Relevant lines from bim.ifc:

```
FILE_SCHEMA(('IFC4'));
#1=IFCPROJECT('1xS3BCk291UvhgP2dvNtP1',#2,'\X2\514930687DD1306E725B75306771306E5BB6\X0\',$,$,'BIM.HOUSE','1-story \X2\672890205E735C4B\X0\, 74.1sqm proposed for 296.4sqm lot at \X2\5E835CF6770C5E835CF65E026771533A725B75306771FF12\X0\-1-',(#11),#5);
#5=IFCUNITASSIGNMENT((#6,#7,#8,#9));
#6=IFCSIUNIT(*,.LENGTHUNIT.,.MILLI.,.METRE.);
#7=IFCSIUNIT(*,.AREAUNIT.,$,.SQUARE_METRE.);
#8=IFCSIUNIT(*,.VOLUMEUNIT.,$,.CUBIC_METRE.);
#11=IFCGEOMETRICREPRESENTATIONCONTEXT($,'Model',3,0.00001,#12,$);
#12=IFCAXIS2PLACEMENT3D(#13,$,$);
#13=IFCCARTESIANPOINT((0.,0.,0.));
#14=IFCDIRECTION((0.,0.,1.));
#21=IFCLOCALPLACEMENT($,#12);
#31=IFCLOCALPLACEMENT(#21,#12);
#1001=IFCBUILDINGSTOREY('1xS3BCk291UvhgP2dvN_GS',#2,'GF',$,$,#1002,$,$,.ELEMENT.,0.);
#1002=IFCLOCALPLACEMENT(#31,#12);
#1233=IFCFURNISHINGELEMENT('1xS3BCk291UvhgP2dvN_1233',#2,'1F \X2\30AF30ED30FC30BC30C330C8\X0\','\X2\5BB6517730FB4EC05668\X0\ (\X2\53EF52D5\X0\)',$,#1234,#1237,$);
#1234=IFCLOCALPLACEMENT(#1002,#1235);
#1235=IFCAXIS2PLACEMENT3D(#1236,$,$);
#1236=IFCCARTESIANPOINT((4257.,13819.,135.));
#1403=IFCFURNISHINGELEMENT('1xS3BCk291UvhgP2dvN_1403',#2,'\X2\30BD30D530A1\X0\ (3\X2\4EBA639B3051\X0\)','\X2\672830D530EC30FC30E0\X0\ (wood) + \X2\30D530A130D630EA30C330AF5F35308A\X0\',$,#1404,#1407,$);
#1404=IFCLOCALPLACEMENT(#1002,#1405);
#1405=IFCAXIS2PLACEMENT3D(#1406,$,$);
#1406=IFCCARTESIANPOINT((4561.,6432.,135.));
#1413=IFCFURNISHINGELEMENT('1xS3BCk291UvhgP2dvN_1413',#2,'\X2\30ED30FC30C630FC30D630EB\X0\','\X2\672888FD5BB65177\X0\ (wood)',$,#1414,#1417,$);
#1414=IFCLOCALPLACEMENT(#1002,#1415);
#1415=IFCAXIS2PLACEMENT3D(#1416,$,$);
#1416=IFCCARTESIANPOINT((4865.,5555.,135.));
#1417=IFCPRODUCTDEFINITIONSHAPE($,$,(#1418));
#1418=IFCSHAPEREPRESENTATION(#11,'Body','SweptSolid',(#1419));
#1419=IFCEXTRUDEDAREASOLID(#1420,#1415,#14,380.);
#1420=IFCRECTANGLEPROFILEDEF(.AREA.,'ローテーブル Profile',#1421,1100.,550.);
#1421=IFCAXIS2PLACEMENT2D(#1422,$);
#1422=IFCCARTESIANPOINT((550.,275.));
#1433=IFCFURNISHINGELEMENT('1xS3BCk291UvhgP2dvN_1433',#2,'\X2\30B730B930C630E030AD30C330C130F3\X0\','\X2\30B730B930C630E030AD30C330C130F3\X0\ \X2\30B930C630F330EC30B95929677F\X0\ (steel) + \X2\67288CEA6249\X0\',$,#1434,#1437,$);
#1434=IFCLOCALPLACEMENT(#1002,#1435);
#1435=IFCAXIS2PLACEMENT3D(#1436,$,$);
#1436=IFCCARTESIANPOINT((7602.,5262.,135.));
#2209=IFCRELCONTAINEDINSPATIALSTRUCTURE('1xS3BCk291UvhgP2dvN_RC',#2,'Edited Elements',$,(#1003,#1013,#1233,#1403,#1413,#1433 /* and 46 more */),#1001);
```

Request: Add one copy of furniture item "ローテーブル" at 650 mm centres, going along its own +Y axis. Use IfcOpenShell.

```python
import ifcopenshell
import ifcopenshell.api.geometry
import ifcopenshell.api.root
import ifcopenshell.util.element
import ifcopenshell.util.placement
import ifcopenshell.util.unit

model = ifcopenshell.open("bim.ifc")
unit_scale = ifcopenshell.util.unit.calculate_unit_scale(model)


def reuse_history(source, copy):
    """copy_class also copies each property set's owner history, people and application; keep the originals."""
    for rel in copy.IsDefinedBy:
        if rel.is_a("IfcRelDefinesByProperties") and (history := rel.RelatingPropertyDefinition.OwnerHistory):
            rel.RelatingPropertyDefinition.OwnerHistory = source.OwnerHistory
            ifcopenshell.util.element.remove_deep2(model, history)


source = model.by_id(1413)
base = ifcopenshell.util.placement.get_local_placement(source.ObjectPlacement)
step = base[:3, 1] * 0.65 / unit_scale

for i in range(1, 2):
    copy = ifcopenshell.api.root.copy_class(model, product=source)
    copy.Representation = ifcopenshell.util.element.copy_deep(
        model, source.Representation, exclude=["IfcGeometricRepresentationContext", "IfcRepresentationMap"]
    )
    reuse_history(source, copy)
    matrix = base.copy()
    matrix[:3, 3] += i * step
    print("added at", matrix[:3, 3].round(3) + 0.0)
    ifcopenshell.api.geometry.edit_object_placement(model, product=copy, matrix=matrix, is_si=False)

model.write("bim_v2.ifc")
```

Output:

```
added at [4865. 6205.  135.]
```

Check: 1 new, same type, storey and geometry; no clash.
